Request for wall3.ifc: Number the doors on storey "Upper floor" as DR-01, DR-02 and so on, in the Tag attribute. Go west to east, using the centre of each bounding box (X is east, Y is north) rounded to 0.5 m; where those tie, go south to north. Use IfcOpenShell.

First a look at what the model holds.

```python
import ifcopenshell
import ifcopenshell.util.element
import ifcopenshell.util.placement

model = ifcopenshell.open("wall3.ifc")
print(model.schema)
storey = next(s for s in model.by_type("IfcBuildingStorey") if s.Name == "Upper floor")
doors = [e for e in ifcopenshell.util.element.get_decomposition(storey) if e.is_a("IfcDoor")]
for e in sorted(doors, key=lambda e: e.id()):
    origin = ifcopenshell.util.placement.get_local_placement(e.ObjectPlacement)[:3, 3]
    print(e.id(), e.Tag, e.Name, origin.round(2) + 0.0, sep=" | ")
```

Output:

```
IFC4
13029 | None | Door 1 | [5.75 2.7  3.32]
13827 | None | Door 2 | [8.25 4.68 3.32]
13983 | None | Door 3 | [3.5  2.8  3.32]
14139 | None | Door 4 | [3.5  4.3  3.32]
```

```python
import ifcopenshell
import ifcopenshell.geom
import ifcopenshell.util.element
import ifcopenshell.util.shape

model = ifcopenshell.open("wall3.ifc")
settings = ifcopenshell.geom.settings()
settings.set("use-world-coords", True)


def centre(element):
    shape = ifcopenshell.geom.create_shape(settings, element)
    return ifcopenshell.util.shape.get_bbox_centroid(shape.geometry)


storey = next(s for s in model.by_type("IfcBuildingStorey") if s.Name == "Upper floor")
doors = [e for e in ifcopenshell.util.element.get_decomposition(storey) if e.is_a("IfcDoor")]

# Insertion points can sit at a corner or the storey origin, so sort by the geometry (in metres).
centres = {e: centre(e) for e in doors}
doors.sort(key=lambda e: (round(centres[e][0] / 0.5), centres[e][1]))

for i, e in enumerate(doors, start=1):
    number = f"DR-{i:02d}"
    e.Tag = number
    print(e.id(), number)

model.write("wall3_rev.ifc")
```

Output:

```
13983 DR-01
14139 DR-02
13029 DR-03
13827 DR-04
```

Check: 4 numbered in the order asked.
